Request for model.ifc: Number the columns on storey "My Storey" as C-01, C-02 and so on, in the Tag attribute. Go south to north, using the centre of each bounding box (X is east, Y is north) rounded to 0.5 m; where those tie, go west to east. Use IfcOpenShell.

First a look at what the model holds.

```python
import ifcopenshell
import ifcopenshell.util.element
import ifcopenshell.util.placement

model = ifcopenshell.open("model.ifc")
print(model.schema)
storey = next(s for s in model.by_type("IfcBuildingStorey") if s.Name == "My Storey")
columns = [e for e in ifcopenshell.util.element.get_decomposition(storey) if e.is_a("IfcColumn")]
for e in sorted(columns, key=lambda e: e.id()):
    origin = ifcopenshell.util.placement.get_local_placement(e.ObjectPlacement)[:3, 3]
    print(e.id(), e.Tag, e.Name, origin.round(2) + 0.0, sep=" | ")
```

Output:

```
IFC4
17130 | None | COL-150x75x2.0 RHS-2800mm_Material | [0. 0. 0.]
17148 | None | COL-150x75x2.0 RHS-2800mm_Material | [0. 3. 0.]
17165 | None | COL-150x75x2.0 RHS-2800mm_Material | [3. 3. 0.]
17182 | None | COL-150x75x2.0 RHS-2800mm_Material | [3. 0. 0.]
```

```python
import ifcopenshell
import ifcopenshell.geom
import ifcopenshell.util.element
import ifcopenshell.util.shape

model = ifcopenshell.open("model.ifc")
settings = ifcopenshell.geom.settings()
settings.set("use-world-coords", True)


def centre(element):
    shape = ifcopenshell.geom.create_shape(settings, element)
    return ifcopenshell.util.shape.get_bbox_centroid(shape.geometry)


storey = next(s for s in model.by_type("IfcBuildingStorey") if s.Name == "My Storey")
columns = [e for e in ifcopenshell.util.element.get_decomposition(storey) if e.is_a("IfcColumn")]

# Insertion points can sit at a corner or the storey origin, so sort by the geometry (in metres).
centres = {e: centre(e) for e in columns}
columns.sort(key=lambda e: (round(centres[e][1] / 0.5), centres[e][0]))

for i, e in enumerate(columns, start=1):
    number = f"C-{i:02d}"
    e.Tag = number
    print(e.id(), number)

model.write("model-out.ifc")
```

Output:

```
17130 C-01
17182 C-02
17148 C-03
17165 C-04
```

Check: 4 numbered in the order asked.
